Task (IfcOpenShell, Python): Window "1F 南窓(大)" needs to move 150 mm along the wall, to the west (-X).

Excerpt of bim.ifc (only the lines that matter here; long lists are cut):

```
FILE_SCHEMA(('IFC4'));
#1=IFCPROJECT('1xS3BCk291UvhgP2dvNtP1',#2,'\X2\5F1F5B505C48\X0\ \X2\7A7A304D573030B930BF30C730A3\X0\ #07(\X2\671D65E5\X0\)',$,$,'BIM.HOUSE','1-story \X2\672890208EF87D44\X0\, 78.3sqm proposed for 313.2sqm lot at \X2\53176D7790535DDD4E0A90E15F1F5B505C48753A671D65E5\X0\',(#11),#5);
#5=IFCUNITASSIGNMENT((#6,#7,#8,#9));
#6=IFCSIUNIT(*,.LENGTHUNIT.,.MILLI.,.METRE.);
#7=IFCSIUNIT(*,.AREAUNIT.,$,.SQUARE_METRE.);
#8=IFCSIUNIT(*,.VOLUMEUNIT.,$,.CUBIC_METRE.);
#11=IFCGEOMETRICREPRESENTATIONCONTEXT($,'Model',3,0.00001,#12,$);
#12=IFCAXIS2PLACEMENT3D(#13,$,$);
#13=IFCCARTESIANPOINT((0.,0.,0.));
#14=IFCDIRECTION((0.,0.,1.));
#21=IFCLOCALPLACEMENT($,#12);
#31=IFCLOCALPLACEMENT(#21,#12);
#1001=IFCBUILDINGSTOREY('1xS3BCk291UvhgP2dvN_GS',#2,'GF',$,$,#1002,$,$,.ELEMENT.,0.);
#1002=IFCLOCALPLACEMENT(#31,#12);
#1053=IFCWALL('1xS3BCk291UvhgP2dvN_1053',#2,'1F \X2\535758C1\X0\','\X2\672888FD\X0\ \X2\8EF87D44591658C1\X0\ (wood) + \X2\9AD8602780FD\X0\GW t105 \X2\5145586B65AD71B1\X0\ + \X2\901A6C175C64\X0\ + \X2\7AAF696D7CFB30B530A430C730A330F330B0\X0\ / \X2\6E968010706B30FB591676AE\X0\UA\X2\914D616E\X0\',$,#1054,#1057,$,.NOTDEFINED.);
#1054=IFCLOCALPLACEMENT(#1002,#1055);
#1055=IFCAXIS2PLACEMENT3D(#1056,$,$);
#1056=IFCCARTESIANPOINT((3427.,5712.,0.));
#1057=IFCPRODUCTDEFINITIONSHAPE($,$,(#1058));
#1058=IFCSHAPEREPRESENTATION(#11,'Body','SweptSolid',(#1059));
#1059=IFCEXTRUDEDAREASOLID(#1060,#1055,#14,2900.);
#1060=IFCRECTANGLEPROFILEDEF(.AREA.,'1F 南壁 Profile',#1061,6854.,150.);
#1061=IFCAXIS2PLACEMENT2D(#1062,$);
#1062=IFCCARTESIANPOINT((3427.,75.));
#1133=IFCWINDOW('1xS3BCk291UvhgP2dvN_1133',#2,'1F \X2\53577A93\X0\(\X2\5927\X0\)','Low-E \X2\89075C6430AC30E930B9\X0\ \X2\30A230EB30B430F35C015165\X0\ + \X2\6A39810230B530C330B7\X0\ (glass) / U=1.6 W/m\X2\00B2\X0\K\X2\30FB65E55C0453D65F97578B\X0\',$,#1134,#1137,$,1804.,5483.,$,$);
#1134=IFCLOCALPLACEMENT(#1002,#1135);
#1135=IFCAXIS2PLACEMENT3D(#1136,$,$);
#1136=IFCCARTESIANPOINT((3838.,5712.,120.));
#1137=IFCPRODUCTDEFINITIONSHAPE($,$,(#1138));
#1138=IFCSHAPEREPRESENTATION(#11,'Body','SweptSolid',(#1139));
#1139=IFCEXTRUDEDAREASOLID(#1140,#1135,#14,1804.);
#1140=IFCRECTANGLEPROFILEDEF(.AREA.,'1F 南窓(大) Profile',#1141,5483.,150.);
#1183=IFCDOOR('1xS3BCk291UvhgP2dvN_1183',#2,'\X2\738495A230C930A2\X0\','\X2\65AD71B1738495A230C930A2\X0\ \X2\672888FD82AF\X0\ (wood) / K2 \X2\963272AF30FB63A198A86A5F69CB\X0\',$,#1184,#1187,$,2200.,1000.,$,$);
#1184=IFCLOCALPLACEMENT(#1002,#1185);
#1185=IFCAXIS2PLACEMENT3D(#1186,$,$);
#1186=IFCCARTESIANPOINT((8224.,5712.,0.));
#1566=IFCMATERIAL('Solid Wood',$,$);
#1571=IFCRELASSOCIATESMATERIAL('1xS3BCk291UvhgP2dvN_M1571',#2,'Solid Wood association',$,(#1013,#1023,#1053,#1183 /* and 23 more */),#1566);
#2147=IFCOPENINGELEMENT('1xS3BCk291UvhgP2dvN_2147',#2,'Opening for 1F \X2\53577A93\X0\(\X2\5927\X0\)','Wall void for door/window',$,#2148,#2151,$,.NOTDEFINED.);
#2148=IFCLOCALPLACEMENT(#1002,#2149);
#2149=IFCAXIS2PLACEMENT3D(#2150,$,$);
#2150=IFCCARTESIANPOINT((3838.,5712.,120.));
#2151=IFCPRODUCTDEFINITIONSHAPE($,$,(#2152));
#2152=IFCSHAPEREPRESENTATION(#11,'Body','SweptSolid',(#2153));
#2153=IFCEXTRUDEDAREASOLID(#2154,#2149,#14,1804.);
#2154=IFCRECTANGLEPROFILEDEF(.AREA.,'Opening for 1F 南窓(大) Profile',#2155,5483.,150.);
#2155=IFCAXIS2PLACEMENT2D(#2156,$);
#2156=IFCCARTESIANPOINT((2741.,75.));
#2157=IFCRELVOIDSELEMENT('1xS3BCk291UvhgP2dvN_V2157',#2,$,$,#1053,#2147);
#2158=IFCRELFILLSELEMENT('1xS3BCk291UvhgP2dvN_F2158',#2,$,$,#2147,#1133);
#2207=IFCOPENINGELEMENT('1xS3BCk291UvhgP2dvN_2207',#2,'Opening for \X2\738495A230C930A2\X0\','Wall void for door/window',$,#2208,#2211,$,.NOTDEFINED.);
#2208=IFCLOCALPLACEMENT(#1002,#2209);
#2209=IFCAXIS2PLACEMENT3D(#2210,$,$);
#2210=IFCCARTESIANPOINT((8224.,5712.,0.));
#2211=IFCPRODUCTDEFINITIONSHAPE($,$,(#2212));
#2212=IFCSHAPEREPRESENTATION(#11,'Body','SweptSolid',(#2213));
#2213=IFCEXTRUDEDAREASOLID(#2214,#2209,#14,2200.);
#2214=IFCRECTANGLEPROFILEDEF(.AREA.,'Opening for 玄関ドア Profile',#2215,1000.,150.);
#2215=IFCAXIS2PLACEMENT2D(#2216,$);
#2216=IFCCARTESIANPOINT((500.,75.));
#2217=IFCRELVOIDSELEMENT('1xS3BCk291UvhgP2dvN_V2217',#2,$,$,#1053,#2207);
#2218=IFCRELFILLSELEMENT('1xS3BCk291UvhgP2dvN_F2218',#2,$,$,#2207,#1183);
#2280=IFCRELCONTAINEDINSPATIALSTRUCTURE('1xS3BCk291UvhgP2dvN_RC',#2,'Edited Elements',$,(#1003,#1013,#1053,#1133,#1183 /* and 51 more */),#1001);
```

```python
import ifcopenshell
import ifcopenshell.api.geometry
import ifcopenshell.util.placement

model = ifcopenshell.open("bim.ifc")

window = model.by_id(1133)
opening = window.FillsVoids[0].RelatingOpeningElement
wall = opening.VoidsElements[0].RelatingBuildingElement

wall_matrix = ifcopenshell.util.placement.get_local_placement(wall.ObjectPlacement)
shift = wall_matrix[:3, 0] * -150.0
before = ifcopenshell.util.placement.get_local_placement(window.ObjectPlacement)[:3, 3].copy()

# The window is not placed relative to its opening, so move both.
for product in (opening, window):
    matrix = ifcopenshell.util.placement.get_local_placement(product.ObjectPlacement)
    matrix[:3, 3] += shift
    ifcopenshell.api.geometry.edit_object_placement(model, product=product, matrix=matrix, is_si=False)

after = ifcopenshell.util.placement.get_local_placement(window.ObjectPlacement)[:3, 3]
print("window moved by", (after - before).round(3) + 0.0)

model.write("bim_rev.ifc")
```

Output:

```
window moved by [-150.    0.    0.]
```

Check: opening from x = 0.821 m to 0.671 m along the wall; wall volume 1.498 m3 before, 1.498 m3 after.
